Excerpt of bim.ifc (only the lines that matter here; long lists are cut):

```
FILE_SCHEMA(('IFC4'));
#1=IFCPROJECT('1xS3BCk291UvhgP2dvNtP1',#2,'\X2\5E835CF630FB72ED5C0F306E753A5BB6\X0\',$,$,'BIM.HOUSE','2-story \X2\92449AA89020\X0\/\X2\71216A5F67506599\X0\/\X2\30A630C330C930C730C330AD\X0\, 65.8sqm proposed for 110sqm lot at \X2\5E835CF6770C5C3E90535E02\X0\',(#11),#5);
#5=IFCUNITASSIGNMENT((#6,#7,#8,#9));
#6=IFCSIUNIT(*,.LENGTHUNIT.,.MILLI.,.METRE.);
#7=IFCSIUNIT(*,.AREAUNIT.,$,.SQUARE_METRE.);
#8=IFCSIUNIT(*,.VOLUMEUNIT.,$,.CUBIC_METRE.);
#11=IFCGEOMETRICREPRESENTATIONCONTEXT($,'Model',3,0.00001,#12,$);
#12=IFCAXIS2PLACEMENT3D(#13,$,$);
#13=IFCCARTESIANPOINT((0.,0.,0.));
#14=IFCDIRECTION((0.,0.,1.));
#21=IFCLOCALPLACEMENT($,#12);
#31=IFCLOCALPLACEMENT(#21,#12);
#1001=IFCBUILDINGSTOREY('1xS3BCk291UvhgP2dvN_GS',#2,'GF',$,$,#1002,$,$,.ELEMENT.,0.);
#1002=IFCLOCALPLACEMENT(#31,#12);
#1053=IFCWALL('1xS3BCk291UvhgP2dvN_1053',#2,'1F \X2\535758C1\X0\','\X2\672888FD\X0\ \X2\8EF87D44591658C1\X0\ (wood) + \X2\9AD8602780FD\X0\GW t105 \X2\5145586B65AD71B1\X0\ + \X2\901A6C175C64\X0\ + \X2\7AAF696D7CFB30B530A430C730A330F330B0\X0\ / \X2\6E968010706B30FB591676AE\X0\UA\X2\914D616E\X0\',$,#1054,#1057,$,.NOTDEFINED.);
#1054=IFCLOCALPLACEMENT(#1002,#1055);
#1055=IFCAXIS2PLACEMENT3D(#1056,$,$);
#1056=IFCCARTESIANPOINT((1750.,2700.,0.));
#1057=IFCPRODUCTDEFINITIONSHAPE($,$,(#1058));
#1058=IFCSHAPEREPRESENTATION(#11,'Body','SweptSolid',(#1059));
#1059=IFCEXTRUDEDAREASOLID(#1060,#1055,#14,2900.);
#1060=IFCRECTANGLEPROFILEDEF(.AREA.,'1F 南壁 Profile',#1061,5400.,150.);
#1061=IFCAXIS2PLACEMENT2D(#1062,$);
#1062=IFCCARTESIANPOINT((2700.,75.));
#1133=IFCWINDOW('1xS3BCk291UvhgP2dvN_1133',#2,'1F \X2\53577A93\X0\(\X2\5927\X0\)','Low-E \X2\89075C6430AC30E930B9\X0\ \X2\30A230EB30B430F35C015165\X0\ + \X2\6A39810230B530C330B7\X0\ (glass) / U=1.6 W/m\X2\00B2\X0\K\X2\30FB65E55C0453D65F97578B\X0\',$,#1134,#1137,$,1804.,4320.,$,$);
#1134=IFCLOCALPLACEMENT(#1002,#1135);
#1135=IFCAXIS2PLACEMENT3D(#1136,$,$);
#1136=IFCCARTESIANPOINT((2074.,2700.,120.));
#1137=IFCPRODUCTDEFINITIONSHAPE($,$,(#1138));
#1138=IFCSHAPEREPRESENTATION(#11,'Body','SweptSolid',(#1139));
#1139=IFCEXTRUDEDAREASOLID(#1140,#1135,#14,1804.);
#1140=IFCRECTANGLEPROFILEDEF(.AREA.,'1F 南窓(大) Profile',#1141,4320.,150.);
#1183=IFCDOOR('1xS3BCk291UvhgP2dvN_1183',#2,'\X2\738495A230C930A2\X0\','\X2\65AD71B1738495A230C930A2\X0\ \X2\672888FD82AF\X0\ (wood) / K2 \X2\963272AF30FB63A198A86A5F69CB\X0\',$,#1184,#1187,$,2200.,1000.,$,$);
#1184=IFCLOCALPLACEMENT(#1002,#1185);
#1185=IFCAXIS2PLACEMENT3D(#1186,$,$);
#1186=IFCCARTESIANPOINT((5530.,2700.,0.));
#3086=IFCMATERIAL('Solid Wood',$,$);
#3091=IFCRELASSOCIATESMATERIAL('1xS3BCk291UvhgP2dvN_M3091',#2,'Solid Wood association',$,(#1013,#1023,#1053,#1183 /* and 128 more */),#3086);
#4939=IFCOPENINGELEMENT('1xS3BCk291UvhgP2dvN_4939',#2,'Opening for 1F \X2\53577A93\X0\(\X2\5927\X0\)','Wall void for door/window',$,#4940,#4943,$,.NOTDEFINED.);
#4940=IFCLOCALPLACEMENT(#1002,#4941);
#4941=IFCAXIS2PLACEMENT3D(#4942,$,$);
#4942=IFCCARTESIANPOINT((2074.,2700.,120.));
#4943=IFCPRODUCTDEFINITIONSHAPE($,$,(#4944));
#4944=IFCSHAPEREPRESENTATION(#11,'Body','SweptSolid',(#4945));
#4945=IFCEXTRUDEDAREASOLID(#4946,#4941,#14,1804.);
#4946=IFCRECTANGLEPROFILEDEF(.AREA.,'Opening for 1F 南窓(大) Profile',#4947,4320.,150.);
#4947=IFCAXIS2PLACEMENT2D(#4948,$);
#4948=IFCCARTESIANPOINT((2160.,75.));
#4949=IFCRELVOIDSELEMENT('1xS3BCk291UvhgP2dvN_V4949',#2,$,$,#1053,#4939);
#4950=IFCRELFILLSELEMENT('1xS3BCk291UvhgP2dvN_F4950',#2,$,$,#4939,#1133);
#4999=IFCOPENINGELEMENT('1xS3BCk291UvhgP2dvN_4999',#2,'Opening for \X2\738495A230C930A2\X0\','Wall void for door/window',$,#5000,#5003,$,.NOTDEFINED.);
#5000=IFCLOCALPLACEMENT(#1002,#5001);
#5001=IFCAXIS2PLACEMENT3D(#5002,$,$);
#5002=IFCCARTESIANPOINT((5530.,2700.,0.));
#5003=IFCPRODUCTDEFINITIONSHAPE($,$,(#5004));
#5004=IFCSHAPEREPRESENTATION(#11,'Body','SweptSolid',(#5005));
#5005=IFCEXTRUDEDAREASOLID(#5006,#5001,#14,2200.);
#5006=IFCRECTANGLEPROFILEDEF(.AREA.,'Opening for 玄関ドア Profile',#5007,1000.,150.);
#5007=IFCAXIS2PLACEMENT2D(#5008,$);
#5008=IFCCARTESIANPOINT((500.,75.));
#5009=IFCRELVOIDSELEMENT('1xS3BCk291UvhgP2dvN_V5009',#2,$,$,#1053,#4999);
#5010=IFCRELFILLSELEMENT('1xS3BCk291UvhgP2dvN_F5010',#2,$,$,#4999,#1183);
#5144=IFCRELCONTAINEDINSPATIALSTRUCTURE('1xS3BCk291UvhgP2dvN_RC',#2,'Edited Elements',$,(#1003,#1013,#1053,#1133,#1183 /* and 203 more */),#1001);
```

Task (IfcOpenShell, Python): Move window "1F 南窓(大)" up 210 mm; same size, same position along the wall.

```python
import numpy as np
import ifcopenshell
import ifcopenshell.api.geometry
import ifcopenshell.util.placement
import ifcopenshell.util.unit

model = ifcopenshell.open("bim.ifc")
unit_scale = ifcopenshell.util.unit.calculate_unit_scale(model)

window = model.by_id(1133)
opening = window.FillsVoids[0].RelatingOpeningElement
dz = 0.21 / unit_scale

shift = np.array([0.0, 0.0, dz])
# The window is not placed relative to its opening, so move both.
for product in (opening, window):
    matrix = ifcopenshell.util.placement.get_local_placement(product.ObjectPlacement)
    matrix[:3, 3] += shift
    ifcopenshell.api.geometry.edit_object_placement(model, product=product, matrix=matrix, is_si=False)

print(f"moved by {dz * unit_scale:+.3f} m")

model.write("bim-out.ifc")
```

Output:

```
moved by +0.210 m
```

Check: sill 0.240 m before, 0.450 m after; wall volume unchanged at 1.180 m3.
